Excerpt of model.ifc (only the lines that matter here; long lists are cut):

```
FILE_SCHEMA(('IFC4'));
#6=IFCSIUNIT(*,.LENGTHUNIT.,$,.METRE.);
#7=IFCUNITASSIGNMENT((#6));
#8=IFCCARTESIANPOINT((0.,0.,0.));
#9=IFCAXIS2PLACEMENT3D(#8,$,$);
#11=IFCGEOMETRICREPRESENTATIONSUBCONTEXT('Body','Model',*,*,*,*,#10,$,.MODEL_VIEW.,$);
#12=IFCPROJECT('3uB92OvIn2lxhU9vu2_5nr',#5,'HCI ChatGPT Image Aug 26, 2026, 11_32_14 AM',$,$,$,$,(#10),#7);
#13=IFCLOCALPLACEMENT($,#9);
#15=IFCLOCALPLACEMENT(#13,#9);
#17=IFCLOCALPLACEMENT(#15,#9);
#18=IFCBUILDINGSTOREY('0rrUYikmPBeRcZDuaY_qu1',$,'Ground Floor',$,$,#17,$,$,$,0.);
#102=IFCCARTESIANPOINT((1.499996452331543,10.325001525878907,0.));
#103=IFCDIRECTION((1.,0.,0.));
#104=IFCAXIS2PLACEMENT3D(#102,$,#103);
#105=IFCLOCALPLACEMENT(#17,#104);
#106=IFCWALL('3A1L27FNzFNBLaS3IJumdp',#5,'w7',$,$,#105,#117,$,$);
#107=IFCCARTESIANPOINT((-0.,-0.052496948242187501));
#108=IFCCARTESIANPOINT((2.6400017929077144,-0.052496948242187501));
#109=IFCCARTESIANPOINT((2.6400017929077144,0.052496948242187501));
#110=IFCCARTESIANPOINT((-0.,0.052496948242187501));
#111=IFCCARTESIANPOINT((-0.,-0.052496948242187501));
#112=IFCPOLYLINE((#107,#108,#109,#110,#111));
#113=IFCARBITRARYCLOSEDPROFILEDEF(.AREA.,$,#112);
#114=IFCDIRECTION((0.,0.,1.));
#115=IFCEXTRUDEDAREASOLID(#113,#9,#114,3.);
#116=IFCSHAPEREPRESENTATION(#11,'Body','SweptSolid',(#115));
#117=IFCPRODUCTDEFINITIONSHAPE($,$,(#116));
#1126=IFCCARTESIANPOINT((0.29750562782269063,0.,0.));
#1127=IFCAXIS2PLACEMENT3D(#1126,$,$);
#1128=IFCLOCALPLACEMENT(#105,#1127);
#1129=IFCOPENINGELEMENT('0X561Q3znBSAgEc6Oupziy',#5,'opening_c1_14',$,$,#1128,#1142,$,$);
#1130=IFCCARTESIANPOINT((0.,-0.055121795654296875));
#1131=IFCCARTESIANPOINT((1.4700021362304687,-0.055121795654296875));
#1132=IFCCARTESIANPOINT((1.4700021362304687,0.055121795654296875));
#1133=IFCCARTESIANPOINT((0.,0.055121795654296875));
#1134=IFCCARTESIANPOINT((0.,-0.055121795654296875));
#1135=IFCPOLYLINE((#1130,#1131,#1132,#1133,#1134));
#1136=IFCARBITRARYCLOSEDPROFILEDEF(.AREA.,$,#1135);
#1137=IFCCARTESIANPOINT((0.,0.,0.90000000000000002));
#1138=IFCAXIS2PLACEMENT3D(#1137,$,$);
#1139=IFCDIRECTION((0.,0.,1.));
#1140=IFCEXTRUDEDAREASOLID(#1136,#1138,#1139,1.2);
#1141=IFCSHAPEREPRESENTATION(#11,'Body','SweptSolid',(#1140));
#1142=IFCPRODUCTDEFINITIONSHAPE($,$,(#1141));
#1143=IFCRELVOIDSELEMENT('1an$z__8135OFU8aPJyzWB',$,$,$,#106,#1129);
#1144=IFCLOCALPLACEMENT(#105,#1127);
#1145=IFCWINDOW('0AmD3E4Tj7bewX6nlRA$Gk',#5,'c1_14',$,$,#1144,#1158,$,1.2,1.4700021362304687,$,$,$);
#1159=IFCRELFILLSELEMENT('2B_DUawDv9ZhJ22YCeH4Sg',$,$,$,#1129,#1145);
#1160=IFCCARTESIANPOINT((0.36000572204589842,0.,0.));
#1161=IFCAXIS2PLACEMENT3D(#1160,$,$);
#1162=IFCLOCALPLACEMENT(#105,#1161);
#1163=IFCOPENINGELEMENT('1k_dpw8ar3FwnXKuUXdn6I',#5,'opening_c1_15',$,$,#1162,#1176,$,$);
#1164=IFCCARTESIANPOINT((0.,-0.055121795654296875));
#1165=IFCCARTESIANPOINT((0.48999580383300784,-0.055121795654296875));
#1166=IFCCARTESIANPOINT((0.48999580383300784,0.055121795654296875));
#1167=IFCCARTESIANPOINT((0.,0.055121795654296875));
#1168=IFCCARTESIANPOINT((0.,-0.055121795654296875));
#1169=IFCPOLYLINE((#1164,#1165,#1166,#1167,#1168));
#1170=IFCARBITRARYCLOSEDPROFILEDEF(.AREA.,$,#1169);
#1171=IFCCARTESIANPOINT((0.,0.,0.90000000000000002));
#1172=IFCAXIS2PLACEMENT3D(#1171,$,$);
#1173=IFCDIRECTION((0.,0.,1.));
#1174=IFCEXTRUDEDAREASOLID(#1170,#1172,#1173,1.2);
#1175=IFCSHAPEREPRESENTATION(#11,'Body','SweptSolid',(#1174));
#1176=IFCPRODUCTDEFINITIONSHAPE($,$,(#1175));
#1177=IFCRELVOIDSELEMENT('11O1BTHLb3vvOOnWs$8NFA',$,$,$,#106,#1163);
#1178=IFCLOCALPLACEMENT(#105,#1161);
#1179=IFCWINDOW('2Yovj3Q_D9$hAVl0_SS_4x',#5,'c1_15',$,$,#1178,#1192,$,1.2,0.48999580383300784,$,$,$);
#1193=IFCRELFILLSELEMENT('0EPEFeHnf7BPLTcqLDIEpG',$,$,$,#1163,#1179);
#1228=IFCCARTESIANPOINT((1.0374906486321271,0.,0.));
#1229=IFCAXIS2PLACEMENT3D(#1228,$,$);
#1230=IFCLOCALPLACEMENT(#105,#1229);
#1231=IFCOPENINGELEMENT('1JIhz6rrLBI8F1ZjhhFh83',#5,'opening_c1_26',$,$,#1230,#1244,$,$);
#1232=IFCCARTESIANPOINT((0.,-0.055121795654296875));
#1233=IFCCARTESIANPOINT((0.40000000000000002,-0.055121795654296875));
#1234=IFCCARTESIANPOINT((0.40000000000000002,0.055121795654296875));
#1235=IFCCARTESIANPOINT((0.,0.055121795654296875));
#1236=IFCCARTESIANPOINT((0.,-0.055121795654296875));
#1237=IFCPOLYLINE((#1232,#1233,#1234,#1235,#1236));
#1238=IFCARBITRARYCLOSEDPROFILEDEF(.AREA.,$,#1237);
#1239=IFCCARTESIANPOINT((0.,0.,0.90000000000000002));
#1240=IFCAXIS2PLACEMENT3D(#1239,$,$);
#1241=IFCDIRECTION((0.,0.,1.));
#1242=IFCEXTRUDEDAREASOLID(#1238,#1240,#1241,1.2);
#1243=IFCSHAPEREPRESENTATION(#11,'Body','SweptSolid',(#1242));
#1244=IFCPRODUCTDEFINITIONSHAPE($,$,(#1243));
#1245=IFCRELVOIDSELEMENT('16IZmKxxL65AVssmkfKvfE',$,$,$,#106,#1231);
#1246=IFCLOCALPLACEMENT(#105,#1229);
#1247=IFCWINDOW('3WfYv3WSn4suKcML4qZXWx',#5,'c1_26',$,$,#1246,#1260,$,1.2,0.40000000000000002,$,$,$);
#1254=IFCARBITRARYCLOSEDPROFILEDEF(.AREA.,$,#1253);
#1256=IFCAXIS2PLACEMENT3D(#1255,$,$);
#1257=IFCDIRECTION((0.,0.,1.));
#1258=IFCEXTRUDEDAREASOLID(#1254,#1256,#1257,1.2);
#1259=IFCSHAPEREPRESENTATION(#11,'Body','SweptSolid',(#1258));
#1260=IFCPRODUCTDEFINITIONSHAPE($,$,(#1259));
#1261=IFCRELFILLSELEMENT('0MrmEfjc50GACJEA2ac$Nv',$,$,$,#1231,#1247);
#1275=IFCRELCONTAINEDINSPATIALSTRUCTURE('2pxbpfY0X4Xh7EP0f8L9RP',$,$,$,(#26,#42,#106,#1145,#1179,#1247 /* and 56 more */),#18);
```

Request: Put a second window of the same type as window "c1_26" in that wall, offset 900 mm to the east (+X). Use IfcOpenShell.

```python
import ifcopenshell
import ifcopenshell.api.feature
import ifcopenshell.api.geometry
import ifcopenshell.api.root
import ifcopenshell.geom
import ifcopenshell.util.element
import ifcopenshell.util.placement
import ifcopenshell.util.shape
import ifcopenshell.util.unit

model = ifcopenshell.open("model.ifc")
unit_scale = ifcopenshell.util.unit.calculate_unit_scale(model)
settings = ifcopenshell.geom.settings()


def volume(element):
    """Net volume in cubic metres, openings subtracted."""
    shape = ifcopenshell.geom.create_shape(settings, element)
    return ifcopenshell.util.shape.get_volume(shape.geometry)


window = model.by_guid("3WfYv3WSn4suKcML4qZXWx")
opening = window.FillsVoids[0].RelatingOpeningElement
wall = opening.VoidsElements[0].RelatingBuildingElement
before = volume(wall)
shift = ifcopenshell.util.placement.get_local_placement(wall.ObjectPlacement)[:3, 0] * 0.9 / unit_scale

# copy_class copies the void relationship, type, container and properties, but no geometry.
new_opening = ifcopenshell.api.root.copy_class(model, product=opening)
new_opening.Representation = ifcopenshell.util.element.copy_deep(
    model, opening.Representation, exclude=["IfcGeometricRepresentationContext", "IfcRepresentationMap"]
)
new_window = ifcopenshell.api.root.copy_class(model, product=window)
new_window.Representation = ifcopenshell.util.element.copy_deep(
    model, window.Representation, exclude=["IfcGeometricRepresentationContext", "IfcRepresentationMap"]
)
ifcopenshell.api.feature.add_filling(model, opening=new_opening, element=new_window)

for old, new in ((opening, new_opening), (window, new_window)):
    matrix = ifcopenshell.util.placement.get_local_placement(old.ObjectPlacement)
    matrix[:3, 3] += shift
    ifcopenshell.api.geometry.edit_object_placement(model, product=new, matrix=matrix, is_si=False)

after = volume(wall)

print(f"wall volume {before:.3f} -> {after:.3f} m3")

model.write("model_edited.ifc")
```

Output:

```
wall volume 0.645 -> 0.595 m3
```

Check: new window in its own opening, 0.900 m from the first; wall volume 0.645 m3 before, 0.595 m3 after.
